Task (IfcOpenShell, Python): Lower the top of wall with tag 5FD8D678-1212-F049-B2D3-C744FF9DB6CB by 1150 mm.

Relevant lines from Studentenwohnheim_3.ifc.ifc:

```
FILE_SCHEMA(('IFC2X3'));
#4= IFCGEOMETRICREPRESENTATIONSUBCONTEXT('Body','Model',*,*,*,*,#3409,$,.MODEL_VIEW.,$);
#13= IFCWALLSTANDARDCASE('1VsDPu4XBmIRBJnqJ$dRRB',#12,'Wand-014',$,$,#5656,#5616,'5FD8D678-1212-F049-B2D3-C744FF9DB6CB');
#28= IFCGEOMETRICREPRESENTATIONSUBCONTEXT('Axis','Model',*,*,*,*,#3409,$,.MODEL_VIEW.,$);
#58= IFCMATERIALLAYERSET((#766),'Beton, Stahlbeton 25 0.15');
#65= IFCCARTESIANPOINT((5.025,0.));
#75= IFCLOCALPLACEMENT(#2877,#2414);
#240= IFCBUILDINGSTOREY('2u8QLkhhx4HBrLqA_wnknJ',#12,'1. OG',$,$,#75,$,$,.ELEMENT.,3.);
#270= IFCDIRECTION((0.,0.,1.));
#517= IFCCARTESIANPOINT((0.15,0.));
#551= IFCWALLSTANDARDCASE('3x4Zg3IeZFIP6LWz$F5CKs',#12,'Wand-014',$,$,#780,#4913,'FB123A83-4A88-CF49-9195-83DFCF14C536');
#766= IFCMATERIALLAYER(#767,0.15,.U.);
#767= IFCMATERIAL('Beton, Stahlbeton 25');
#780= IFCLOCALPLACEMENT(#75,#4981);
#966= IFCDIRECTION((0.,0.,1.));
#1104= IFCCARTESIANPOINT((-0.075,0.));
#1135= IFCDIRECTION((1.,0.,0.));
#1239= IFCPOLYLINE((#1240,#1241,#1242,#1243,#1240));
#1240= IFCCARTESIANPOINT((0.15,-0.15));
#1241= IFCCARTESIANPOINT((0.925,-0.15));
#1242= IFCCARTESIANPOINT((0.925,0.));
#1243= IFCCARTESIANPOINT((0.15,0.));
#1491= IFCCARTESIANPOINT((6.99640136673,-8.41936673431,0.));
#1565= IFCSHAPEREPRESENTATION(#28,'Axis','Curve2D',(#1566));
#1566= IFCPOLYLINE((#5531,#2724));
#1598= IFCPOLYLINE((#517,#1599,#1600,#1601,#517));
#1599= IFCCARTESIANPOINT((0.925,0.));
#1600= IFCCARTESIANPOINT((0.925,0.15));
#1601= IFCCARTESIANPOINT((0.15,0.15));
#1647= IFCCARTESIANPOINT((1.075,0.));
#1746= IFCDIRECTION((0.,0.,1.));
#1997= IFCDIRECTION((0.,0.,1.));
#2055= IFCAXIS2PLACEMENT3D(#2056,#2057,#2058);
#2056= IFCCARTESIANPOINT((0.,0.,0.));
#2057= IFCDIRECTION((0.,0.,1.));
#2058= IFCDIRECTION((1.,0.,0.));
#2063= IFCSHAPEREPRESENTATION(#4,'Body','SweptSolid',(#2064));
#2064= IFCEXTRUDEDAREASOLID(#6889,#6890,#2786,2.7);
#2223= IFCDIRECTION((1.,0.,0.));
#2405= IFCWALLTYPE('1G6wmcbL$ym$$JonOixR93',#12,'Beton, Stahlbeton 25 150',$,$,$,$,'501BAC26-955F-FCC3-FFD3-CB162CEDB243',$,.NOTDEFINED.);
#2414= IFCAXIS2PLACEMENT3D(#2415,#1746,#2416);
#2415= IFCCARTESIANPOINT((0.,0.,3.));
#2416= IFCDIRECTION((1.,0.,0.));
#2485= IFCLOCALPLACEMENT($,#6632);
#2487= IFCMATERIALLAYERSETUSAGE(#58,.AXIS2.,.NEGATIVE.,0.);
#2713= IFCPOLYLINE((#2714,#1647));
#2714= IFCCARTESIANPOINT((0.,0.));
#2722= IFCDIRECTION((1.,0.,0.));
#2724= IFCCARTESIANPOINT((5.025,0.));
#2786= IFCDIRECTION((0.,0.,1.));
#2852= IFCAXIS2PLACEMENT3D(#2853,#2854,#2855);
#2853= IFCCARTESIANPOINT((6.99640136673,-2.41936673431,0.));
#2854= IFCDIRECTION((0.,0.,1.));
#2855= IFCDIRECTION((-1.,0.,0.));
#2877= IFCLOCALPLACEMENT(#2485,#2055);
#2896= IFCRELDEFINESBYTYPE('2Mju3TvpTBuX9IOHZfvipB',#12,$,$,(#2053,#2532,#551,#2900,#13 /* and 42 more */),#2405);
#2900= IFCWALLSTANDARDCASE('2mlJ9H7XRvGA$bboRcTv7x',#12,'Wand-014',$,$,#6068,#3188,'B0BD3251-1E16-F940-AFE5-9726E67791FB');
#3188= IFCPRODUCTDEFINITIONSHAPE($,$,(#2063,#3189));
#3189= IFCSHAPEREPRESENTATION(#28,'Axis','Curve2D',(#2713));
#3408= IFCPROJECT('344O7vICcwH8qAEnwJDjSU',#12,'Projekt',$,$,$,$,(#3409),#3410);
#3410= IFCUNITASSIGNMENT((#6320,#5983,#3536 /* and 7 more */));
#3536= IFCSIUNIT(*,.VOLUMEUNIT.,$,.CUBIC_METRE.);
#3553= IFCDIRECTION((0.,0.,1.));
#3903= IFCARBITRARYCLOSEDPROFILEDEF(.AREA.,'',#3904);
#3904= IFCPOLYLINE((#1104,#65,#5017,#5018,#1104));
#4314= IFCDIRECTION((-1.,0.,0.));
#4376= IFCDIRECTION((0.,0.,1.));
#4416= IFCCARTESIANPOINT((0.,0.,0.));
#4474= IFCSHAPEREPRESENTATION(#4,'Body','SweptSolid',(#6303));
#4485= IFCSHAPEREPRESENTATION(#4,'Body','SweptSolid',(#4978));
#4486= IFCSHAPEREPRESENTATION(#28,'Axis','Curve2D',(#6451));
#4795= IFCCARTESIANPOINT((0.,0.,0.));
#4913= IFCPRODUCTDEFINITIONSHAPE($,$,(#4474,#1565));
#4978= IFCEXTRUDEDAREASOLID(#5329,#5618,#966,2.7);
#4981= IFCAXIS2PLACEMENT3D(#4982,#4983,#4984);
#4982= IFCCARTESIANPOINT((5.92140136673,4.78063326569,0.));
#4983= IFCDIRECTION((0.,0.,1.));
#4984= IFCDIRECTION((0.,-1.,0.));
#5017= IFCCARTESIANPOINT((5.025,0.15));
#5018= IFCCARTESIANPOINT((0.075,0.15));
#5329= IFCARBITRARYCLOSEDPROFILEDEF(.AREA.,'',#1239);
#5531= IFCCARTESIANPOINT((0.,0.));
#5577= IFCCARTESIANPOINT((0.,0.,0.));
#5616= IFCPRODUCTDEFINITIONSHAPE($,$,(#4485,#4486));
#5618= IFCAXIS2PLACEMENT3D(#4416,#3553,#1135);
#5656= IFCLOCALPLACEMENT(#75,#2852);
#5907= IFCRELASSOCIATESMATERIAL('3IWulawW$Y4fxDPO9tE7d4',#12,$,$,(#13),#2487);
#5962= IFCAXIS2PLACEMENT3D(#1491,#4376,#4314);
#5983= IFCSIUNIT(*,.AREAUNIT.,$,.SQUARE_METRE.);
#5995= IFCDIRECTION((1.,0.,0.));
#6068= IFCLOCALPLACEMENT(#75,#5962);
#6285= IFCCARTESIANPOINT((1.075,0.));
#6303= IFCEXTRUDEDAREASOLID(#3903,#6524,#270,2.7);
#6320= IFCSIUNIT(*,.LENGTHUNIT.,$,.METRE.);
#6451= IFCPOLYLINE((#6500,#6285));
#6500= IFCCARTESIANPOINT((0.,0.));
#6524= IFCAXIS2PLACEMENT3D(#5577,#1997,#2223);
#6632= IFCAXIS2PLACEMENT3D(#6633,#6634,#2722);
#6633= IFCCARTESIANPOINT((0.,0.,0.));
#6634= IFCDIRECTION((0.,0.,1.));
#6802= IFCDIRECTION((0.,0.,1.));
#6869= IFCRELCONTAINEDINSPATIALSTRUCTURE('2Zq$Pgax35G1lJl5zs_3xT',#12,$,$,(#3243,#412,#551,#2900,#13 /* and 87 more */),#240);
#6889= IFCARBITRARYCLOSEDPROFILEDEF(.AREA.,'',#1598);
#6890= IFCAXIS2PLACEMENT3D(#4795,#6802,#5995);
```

```python
import ifcopenshell
import ifcopenshell.geom
import ifcopenshell.util.representation
import ifcopenshell.util.shape
import ifcopenshell.util.unit

model = ifcopenshell.open("Studentenwohnheim_3.ifc.ifc")
unit_scale = ifcopenshell.util.unit.calculate_unit_scale(model)
settings = ifcopenshell.geom.settings()


def volume(element):
    """Net volume in cubic metres, openings subtracted."""
    shape = ifcopenshell.geom.create_shape(settings, element)
    return ifcopenshell.util.shape.get_volume(shape.geometry)


wall = model.by_guid("1VsDPu4XBmIRBJnqJ$dRRB")
before = volume(wall)

body = ifcopenshell.util.representation.get_representation(wall, "Model", "Body")
solid = body.Items[0]
old_height = solid.Depth
solid.Depth -= 1.15 / unit_scale
after = volume(wall)

print(f"height {old_height:g} -> {solid.Depth:g}, volume {before:.3f} -> {after:.3f} m3")

model.write("Studentenwohnheim_3.ifc_updated.ifc")
```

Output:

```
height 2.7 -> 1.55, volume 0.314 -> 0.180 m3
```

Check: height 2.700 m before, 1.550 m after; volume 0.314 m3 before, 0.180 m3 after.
